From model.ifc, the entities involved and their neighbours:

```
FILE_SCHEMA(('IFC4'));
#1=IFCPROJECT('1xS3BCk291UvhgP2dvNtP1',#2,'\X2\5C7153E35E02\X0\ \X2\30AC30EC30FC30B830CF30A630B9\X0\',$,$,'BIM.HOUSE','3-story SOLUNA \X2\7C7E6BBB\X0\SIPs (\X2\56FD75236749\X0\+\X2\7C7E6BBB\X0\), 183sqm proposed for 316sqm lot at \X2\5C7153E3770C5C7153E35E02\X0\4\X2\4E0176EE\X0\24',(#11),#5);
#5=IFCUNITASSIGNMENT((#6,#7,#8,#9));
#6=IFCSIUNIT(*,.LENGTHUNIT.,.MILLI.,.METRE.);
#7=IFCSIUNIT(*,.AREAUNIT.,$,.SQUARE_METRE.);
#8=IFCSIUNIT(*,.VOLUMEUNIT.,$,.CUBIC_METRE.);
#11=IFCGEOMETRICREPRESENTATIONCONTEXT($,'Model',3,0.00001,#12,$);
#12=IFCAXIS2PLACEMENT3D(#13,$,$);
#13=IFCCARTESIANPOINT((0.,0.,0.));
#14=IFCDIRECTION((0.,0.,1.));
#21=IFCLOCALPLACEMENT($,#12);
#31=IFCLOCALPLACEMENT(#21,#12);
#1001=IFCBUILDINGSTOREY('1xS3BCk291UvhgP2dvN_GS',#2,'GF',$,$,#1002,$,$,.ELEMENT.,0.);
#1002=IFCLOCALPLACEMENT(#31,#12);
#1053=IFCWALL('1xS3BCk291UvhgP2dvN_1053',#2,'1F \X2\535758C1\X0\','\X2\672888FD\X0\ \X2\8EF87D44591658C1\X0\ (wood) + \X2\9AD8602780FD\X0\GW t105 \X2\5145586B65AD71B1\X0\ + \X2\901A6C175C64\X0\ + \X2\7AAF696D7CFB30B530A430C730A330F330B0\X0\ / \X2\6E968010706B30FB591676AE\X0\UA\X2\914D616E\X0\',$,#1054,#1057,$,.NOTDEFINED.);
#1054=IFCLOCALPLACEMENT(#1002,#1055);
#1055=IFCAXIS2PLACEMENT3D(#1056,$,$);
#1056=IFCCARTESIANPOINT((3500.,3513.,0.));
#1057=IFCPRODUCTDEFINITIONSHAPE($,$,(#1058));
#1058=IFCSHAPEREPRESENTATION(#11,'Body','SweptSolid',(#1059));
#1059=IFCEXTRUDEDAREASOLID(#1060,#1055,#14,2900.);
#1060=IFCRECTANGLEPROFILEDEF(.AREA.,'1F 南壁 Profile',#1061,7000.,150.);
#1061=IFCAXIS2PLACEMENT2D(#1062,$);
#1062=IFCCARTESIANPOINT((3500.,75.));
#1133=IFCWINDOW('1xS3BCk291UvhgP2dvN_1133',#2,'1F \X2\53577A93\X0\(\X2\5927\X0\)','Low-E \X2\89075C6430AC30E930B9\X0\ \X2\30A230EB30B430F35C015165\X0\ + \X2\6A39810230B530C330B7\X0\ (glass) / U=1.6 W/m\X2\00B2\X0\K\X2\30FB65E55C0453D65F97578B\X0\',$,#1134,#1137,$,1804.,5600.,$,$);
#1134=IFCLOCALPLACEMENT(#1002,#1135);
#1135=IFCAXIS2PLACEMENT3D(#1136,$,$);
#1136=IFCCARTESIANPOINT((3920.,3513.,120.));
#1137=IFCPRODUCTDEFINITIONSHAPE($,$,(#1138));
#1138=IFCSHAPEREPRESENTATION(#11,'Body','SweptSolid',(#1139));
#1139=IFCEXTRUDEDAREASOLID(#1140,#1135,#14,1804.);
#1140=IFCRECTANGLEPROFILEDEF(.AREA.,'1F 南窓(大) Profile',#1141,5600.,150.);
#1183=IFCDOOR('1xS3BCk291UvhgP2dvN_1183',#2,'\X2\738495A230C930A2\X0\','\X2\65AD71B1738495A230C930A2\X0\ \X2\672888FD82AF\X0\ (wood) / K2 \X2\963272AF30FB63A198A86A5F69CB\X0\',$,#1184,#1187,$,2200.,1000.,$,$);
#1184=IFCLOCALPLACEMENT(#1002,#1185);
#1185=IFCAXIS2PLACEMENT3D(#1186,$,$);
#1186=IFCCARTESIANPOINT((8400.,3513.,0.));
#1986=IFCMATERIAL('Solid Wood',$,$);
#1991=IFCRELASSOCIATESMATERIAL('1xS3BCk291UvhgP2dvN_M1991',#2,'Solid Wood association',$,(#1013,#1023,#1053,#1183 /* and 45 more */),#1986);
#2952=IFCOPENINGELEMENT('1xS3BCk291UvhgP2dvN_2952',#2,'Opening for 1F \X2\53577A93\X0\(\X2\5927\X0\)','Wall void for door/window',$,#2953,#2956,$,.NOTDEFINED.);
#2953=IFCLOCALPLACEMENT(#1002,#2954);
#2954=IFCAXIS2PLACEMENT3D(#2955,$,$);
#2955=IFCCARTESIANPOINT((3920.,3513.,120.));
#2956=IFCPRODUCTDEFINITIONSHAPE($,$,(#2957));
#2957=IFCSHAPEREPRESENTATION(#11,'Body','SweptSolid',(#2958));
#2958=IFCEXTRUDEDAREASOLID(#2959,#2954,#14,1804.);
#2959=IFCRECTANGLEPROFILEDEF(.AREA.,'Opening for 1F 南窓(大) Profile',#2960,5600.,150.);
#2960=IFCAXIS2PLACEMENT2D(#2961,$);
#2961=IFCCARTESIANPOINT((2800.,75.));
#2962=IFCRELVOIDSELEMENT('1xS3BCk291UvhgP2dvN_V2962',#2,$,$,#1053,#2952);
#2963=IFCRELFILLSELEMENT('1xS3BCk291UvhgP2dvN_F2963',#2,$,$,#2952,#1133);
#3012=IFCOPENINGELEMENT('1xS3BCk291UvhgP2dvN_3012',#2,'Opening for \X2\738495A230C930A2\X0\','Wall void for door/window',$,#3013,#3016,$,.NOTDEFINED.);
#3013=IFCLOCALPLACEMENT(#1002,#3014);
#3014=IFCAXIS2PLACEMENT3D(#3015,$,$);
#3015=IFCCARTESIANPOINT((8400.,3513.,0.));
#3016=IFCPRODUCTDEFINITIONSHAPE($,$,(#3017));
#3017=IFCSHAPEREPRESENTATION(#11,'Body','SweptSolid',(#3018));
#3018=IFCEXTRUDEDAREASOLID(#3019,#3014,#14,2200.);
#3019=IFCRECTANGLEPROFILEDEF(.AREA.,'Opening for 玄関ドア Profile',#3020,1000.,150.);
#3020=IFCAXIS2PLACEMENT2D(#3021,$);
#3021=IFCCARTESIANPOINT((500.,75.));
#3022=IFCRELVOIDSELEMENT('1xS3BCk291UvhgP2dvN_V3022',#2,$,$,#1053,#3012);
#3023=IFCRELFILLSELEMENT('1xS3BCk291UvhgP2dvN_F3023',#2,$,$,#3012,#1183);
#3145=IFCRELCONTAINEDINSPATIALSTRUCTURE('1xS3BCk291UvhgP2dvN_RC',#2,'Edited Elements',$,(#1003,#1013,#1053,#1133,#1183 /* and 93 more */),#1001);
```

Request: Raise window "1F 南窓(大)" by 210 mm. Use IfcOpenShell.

```python
import numpy as np
import ifcopenshell
import ifcopenshell.api.geometry
import ifcopenshell.util.placement
import ifcopenshell.util.unit

model = ifcopenshell.open("model.ifc")
unit_scale = ifcopenshell.util.unit.calculate_unit_scale(model)

window = model.by_id(1133)
opening = window.FillsVoids[0].RelatingOpeningElement
dz = 210.0

shift = np.array([0.0, 0.0, dz])
# The window is not placed relative to its opening, so move both.
for product in (opening, window):
    matrix = ifcopenshell.util.placement.get_local_placement(product.ObjectPlacement)
    matrix[:3, 3] += shift
    ifcopenshell.api.geometry.edit_object_placement(model, product=product, matrix=matrix, is_si=False)

print(f"moved by {dz * unit_scale:+.3f} m")

model.write("model_rev.ifc")
```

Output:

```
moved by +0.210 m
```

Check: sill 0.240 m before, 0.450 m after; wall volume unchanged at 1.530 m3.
